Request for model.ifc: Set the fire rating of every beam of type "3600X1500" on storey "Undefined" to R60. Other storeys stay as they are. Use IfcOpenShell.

First a look at what the model holds.

```python
import ifcopenshell
import ifcopenshell.util.element

model = ifcopenshell.open("model.ifc")
print(model.schema)
storey = next(s for s in model.by_type("IfcBuildingStorey") if s.Name == "Undefined")
beams = [e for e in ifcopenshell.util.element.get_decomposition(storey) if e.is_a("IfcBeam")]
seen = {}
for e in beams:
    element_type = ifcopenshell.util.element.get_type(e)
    key = (element_type.Name if element_type != e and element_type else None, ifcopenshell.util.element.get_pset(e, "Pset_BeamCommon", "FireRating"))
    seen[key] = seen.get(key, 0) + 1
for (name, value), count in sorted(seen.items(), key=str):
    print(count, "x", name, "|", value)
```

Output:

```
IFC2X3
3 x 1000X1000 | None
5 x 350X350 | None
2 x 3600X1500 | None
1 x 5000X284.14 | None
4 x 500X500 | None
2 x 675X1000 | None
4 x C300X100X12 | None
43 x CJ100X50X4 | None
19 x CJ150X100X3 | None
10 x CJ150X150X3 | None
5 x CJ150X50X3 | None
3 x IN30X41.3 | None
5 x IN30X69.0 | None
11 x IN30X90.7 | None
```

```python
import ifcopenshell
import ifcopenshell.api.pset
import ifcopenshell.util.element

model = ifcopenshell.open("model.ifc")

storey = next(s for s in model.by_type("IfcBuildingStorey") if s.Name == "Undefined")
beams = [e for e in ifcopenshell.util.element.get_decomposition(storey) if e.is_a("IfcBeam")]

count = 0
for e in beams:
    element_type = ifcopenshell.util.element.get_type(e)
    if element_type in (None, e) or element_type.Name != "3600X1500":
        continue
    # add_pset returns the element's existing set when there is one.
    pset = ifcopenshell.api.pset.add_pset(model, product=e, name="Pset_BeamCommon")
    ifcopenshell.api.pset.edit_pset(model, pset=pset, properties={"FireRating": "R60"})
    count += 1

print(count, "beams updated")

model.write("model_rev.ifc")
```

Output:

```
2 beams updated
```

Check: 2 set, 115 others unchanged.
